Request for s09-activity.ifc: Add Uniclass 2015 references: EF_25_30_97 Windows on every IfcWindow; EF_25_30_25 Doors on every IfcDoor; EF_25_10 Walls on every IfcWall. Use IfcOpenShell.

First a look at what the model holds.

```python
import ifcopenshell

model = ifcopenshell.open("s09-activity.ifc")
print(model.schema)
print("classifications:", [c.Name for c in model.by_type("IfcClassification")])
for ifc_class in ("IfcDoor", "IfcRoof", "IfcStair", "IfcWall", "IfcWindow"):
    print(ifc_class, len(model.by_type(ifc_class)))
```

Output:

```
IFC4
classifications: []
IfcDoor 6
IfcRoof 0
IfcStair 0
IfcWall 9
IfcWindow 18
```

```python
import ifcopenshell
import ifcopenshell.api.classification

model = ifcopenshell.open("s09-activity.ifc")

system = ifcopenshell.api.classification.add_classification(model, classification="Uniclass 2015")

codes = {
    "IfcWindow": ("EF_25_30_97", "Windows"),
    "IfcDoor": ("EF_25_30_25", "Doors"),
    "IfcWall": ("EF_25_10", "Walls"),
}
for ifc_class, (code, name) in codes.items():
    products = model.by_type(ifc_class)
    ifcopenshell.api.classification.add_reference(
        model, products=products, classification=system, identification=code, name=name
    )
    print(code, len(products))

model.write("s09-activity_rev.ifc")
```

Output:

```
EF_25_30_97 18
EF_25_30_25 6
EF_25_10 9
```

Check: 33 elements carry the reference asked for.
